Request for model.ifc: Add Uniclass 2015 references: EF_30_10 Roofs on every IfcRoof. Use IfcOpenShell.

First a look at what the model holds.

```python
import ifcopenshell

model = ifcopenshell.open("model.ifc")
print(model.schema)
print("classifications:", [c.Name for c in model.by_type("IfcClassification")])
for ifc_class in ("IfcDoor", "IfcRoof", "IfcStair", "IfcWall", "IfcWindow"):
    print(ifc_class, len(model.by_type(ifc_class)))
```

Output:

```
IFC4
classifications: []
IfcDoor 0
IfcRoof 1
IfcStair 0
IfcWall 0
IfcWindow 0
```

```python
import ifcopenshell
import ifcopenshell.api.classification

model = ifcopenshell.open("model.ifc")

system = ifcopenshell.api.classification.add_classification(model, classification="Uniclass 2015")

codes = {
    "IfcRoof": ("EF_30_10", "Roofs"),
}
for ifc_class, (code, name) in codes.items():
    products = model.by_type(ifc_class)
    ifcopenshell.api.classification.add_reference(
        model, products=products, classification=system, identification=code, name=name
    )
    print(code, len(products))

model.write("model_rev.ifc")
```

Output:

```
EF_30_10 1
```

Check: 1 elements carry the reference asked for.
